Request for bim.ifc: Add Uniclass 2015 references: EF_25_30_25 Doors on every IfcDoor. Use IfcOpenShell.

First a look at what the model holds.

```python
import ifcopenshell

model = ifcopenshell.open("bim.ifc")
print(model.schema)
print("classifications:", [c.Name for c in model.by_type("IfcClassification")])
for ifc_class in ("IfcDoor", "IfcRoof", "IfcStair", "IfcWall", "IfcWindow"):
    print(ifc_class, len(model.by_type(ifc_class)))
```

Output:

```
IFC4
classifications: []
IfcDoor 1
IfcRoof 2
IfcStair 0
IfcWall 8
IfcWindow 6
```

```python
import ifcopenshell
import ifcopenshell.api.classification

model = ifcopenshell.open("bim.ifc")

system = ifcopenshell.api.classification.add_classification(model, classification="Uniclass 2015")

codes = {
    "IfcDoor": ("EF_25_30_25", "Doors"),
}
for ifc_class, (code, name) in codes.items():
    products = model.by_type(ifc_class)
    ifcopenshell.api.classification.add_reference(
        model, products=products, classification=system, identification=code, name=name
    )
    print(code, len(products))

model.write("bim-out.ifc")
```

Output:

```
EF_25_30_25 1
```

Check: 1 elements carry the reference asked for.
